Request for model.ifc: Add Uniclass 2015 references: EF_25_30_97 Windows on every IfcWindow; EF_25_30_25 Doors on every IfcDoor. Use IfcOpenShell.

First a look at what the model holds.

```python
import ifcopenshell

model = ifcopenshell.open("model.ifc")
print(model.schema)
print("classifications:", [c.Name for c in model.by_type("IfcClassification")])
for ifc_class in ("IfcDoor", "IfcRoof", "IfcStair", "IfcWall", "IfcWindow"):
    print(ifc_class, len(model.by_type(ifc_class)))
```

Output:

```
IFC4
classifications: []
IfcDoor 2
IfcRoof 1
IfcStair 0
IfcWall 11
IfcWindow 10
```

```python
import ifcopenshell
import ifcopenshell.api.classification

model = ifcopenshell.open("model.ifc")

system = ifcopenshell.api.classification.add_classification(model, classification="Uniclass 2015")

codes = {
    "IfcWindow": ("EF_25_30_97", "Windows"),
    "IfcDoor": ("EF_25_30_25", "Doors"),
}
for ifc_class, (code, name) in codes.items():
    products = model.by_type(ifc_class)
    ifcopenshell.api.classification.add_reference(
        model, products=products, classification=system, identification=code, name=name
    )
    print(code, len(products))

model.write("model_updated.ifc")
```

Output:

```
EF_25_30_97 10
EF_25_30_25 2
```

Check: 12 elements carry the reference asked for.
